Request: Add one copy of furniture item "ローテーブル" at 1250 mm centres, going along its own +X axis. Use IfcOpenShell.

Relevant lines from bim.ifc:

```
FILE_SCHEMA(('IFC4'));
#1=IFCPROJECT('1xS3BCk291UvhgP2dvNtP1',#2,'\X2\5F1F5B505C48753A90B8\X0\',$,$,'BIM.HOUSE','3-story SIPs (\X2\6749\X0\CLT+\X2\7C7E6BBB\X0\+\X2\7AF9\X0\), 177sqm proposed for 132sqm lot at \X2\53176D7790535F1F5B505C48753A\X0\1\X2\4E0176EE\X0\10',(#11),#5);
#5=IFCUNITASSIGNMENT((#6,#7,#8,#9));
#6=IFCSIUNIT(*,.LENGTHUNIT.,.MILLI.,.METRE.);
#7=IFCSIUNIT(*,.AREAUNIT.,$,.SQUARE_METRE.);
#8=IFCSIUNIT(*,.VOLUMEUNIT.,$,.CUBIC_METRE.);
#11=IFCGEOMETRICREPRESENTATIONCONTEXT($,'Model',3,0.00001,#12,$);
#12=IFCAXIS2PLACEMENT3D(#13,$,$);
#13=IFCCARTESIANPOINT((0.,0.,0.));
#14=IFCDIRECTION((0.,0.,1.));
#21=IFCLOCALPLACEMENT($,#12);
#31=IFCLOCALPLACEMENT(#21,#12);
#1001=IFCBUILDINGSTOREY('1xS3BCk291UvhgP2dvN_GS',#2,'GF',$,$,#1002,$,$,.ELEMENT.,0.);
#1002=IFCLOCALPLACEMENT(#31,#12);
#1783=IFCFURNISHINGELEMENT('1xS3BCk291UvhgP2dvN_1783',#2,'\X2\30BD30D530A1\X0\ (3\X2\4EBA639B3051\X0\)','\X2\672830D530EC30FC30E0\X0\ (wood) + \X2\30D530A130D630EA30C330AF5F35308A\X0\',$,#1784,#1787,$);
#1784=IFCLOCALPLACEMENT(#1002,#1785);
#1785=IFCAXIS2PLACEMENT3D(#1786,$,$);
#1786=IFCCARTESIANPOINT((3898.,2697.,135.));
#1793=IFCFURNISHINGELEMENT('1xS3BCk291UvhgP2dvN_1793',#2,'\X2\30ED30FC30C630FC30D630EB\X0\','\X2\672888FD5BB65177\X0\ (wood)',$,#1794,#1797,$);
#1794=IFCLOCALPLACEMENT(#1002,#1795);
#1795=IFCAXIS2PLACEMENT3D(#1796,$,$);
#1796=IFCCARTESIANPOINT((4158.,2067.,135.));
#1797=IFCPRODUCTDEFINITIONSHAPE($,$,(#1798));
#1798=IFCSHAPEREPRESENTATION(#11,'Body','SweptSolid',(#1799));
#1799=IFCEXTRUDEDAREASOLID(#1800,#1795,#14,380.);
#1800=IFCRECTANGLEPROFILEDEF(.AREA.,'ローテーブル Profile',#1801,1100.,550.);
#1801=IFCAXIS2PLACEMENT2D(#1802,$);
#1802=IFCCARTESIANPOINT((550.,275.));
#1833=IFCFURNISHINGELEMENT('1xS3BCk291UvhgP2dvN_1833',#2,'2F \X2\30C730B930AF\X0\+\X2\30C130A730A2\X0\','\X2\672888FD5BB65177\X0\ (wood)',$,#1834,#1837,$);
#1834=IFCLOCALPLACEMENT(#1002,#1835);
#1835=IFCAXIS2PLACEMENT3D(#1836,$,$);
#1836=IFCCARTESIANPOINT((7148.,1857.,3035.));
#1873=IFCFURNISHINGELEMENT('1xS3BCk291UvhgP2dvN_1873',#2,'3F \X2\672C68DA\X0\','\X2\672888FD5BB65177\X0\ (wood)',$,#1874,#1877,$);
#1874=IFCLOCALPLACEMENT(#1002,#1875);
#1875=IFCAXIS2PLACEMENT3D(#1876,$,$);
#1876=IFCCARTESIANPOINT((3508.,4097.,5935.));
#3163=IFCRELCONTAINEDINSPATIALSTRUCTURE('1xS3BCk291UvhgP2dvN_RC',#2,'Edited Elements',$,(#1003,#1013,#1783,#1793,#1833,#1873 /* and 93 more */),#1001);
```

```python
import ifcopenshell
import ifcopenshell.api.geometry
import ifcopenshell.api.root
import ifcopenshell.util.element
import ifcopenshell.util.placement
import ifcopenshell.util.unit

model = ifcopenshell.open("bim.ifc")
unit_scale = ifcopenshell.util.unit.calculate_unit_scale(model)


def reuse_history(source, copy):
    """copy_class also copies each property set's owner history, people and application; keep the originals."""
    for rel in copy.IsDefinedBy:
        if rel.is_a("IfcRelDefinesByProperties") and (history := rel.RelatingPropertyDefinition.OwnerHistory):
            rel.RelatingPropertyDefinition.OwnerHistory = source.OwnerHistory
            ifcopenshell.util.element.remove_deep2(model, history)


source = model.by_id(1793)
base = ifcopenshell.util.placement.get_local_placement(source.ObjectPlacement)
step = base[:3, 0] * 1.25 / unit_scale

for i in range(1, 2):
    copy = ifcopenshell.api.root.copy_class(model, product=source)
    copy.Representation = ifcopenshell.util.element.copy_deep(
        model, source.Representation, exclude=["IfcGeometricRepresentationContext", "IfcRepresentationMap"]
    )
    reuse_history(source, copy)
    matrix = base.copy()
    matrix[:3, 3] += i * step
    print("added at", matrix[:3, 3].round(3) + 0.0)
    ifcopenshell.api.geometry.edit_object_placement(model, product=copy, matrix=matrix, is_si=False)

model.write("bim_rev.ifc")
```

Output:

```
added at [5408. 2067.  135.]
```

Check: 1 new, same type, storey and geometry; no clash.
